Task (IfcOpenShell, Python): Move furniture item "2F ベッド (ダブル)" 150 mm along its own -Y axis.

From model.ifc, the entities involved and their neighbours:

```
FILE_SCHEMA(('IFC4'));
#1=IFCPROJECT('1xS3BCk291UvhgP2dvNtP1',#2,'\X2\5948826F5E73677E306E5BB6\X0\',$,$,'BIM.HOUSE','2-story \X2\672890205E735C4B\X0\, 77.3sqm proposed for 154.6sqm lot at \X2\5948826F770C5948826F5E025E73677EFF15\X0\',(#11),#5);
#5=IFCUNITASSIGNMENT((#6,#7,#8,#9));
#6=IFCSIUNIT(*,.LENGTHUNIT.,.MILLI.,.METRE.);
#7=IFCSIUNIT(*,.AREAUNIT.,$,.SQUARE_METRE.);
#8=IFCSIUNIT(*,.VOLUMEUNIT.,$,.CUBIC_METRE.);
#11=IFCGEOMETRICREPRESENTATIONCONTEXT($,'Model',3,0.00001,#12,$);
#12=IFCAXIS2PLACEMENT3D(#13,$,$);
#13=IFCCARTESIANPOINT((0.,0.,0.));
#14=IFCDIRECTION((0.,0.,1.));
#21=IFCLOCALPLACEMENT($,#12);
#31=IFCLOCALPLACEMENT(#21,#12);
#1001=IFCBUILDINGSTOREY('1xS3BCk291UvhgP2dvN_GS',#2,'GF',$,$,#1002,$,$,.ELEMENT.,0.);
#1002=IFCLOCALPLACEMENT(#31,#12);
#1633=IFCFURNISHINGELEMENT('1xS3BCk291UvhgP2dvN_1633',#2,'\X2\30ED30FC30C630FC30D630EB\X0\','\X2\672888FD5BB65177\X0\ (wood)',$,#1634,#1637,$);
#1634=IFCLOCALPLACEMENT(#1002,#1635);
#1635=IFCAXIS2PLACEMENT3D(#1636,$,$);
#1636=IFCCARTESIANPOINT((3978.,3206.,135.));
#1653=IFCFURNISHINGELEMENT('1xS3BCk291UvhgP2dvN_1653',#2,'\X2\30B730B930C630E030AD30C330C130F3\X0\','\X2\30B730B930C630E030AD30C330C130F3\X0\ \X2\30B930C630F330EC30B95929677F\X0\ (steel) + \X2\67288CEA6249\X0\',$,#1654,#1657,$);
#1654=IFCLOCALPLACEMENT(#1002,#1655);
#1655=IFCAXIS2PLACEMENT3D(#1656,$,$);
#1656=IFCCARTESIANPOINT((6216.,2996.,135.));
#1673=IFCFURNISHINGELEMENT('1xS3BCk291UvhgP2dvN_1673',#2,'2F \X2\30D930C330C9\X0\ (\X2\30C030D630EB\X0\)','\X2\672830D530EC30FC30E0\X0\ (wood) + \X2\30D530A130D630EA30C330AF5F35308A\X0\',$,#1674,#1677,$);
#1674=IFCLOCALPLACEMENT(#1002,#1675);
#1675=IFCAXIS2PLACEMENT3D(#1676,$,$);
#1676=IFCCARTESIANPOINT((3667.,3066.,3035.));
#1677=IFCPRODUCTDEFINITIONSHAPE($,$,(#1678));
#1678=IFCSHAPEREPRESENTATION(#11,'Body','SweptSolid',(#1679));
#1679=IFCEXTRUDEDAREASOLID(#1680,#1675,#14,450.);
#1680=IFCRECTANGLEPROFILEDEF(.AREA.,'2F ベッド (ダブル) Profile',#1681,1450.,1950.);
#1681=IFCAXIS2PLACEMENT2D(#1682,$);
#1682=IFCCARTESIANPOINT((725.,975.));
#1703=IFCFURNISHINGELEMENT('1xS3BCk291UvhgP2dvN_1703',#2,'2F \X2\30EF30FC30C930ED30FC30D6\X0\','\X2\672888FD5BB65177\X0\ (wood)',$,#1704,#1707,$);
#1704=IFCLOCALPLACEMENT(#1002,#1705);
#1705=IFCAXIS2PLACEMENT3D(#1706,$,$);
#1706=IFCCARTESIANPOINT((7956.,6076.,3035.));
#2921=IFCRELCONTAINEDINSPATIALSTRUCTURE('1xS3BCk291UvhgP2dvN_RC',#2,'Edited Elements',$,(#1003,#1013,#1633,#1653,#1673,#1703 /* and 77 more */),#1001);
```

```python
import ifcopenshell
import ifcopenshell.api.geometry
import ifcopenshell.util.placement
import ifcopenshell.util.unit

model = ifcopenshell.open("model.ifc")
unit_scale = ifcopenshell.util.unit.calculate_unit_scale(model)

item = model.by_guid("1xS3BCk291UvhgP2dvN_1673")
matrix = ifcopenshell.util.placement.get_local_placement(item.ObjectPlacement)
matrix[:3, 3] -= matrix[:3, 1] * 0.15 / unit_scale
ifcopenshell.api.geometry.edit_object_placement(model, product=item, matrix=matrix, is_si=False)

print(ifcopenshell.util.placement.get_local_placement(item.ObjectPlacement).round(3) + 0.0)

model.write("model_rev.ifc")
```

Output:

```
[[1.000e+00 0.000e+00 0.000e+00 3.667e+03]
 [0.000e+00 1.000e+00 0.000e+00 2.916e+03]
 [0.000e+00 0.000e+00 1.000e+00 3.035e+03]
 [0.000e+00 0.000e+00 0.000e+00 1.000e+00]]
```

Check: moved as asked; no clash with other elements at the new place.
